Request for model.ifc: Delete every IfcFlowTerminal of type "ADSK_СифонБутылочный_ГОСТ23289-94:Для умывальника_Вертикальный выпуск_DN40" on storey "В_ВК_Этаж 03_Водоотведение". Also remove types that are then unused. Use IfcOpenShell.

First a look at what the model holds.

```python
import ifcopenshell
import ifcopenshell.util.element

model = ifcopenshell.open("model.ifc")
print(model.schema)
storey = next(s for s in model.by_type("IfcBuildingStorey") if s.Name == "В_ВК_Этаж 03_Водоотведение")
terminals = [e for e in ifcopenshell.util.element.get_decomposition(storey) if e.is_a("IfcFlowTerminal")]
seen = {}
for e in terminals:
    element_type = ifcopenshell.util.element.get_type(e)
    name = element_type.Name if element_type not in (None, e) else None
    seen[name] = seen.get(name, 0) + 1
for name, count in sorted(seen.items(), key=str):
    print(count, "x", name)
```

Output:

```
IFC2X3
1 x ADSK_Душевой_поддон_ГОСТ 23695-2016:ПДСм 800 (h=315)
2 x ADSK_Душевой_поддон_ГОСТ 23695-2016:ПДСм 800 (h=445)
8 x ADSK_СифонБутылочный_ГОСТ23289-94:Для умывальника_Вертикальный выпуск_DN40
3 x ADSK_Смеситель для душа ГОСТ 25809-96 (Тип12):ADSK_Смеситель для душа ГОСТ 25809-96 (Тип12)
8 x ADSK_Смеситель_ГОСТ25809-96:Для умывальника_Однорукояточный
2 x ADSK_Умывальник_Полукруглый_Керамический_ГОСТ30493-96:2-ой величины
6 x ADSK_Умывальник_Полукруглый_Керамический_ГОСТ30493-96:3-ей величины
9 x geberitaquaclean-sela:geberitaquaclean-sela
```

```python
import ifcopenshell
import ifcopenshell.api.root
import ifcopenshell.util.element

model = ifcopenshell.open("model.ifc")

storey = next(s for s in model.by_type("IfcBuildingStorey") if s.Name == "В_ВК_Этаж 03_Водоотведение")
terminals = [e for e in ifcopenshell.util.element.get_decomposition(storey) if e.is_a("IfcFlowTerminal")]
targets = [e for e in terminals if (t := ifcopenshell.util.element.get_type(e)) not in (None, e) and t.Name == "ADSK_СифонБутылочный_ГОСТ23289-94:Для умывальника_Вертикальный выпуск_DN40"]
types = {ifcopenshell.util.element.get_type(e) for e in targets} - {None, *targets}

for e in targets:
    ifcopenshell.api.root.remove_product(model, product=e)
print(len(targets), "removed")

unused = [t for t in types if not ifcopenshell.util.element.get_types(t)]
for t in unused:
    ifcopenshell.api.root.remove_product(model, product=t)
print(len(unused), "unused types removed")

model.write("model_v2.ifc")
```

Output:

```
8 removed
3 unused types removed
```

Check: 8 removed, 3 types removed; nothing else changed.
